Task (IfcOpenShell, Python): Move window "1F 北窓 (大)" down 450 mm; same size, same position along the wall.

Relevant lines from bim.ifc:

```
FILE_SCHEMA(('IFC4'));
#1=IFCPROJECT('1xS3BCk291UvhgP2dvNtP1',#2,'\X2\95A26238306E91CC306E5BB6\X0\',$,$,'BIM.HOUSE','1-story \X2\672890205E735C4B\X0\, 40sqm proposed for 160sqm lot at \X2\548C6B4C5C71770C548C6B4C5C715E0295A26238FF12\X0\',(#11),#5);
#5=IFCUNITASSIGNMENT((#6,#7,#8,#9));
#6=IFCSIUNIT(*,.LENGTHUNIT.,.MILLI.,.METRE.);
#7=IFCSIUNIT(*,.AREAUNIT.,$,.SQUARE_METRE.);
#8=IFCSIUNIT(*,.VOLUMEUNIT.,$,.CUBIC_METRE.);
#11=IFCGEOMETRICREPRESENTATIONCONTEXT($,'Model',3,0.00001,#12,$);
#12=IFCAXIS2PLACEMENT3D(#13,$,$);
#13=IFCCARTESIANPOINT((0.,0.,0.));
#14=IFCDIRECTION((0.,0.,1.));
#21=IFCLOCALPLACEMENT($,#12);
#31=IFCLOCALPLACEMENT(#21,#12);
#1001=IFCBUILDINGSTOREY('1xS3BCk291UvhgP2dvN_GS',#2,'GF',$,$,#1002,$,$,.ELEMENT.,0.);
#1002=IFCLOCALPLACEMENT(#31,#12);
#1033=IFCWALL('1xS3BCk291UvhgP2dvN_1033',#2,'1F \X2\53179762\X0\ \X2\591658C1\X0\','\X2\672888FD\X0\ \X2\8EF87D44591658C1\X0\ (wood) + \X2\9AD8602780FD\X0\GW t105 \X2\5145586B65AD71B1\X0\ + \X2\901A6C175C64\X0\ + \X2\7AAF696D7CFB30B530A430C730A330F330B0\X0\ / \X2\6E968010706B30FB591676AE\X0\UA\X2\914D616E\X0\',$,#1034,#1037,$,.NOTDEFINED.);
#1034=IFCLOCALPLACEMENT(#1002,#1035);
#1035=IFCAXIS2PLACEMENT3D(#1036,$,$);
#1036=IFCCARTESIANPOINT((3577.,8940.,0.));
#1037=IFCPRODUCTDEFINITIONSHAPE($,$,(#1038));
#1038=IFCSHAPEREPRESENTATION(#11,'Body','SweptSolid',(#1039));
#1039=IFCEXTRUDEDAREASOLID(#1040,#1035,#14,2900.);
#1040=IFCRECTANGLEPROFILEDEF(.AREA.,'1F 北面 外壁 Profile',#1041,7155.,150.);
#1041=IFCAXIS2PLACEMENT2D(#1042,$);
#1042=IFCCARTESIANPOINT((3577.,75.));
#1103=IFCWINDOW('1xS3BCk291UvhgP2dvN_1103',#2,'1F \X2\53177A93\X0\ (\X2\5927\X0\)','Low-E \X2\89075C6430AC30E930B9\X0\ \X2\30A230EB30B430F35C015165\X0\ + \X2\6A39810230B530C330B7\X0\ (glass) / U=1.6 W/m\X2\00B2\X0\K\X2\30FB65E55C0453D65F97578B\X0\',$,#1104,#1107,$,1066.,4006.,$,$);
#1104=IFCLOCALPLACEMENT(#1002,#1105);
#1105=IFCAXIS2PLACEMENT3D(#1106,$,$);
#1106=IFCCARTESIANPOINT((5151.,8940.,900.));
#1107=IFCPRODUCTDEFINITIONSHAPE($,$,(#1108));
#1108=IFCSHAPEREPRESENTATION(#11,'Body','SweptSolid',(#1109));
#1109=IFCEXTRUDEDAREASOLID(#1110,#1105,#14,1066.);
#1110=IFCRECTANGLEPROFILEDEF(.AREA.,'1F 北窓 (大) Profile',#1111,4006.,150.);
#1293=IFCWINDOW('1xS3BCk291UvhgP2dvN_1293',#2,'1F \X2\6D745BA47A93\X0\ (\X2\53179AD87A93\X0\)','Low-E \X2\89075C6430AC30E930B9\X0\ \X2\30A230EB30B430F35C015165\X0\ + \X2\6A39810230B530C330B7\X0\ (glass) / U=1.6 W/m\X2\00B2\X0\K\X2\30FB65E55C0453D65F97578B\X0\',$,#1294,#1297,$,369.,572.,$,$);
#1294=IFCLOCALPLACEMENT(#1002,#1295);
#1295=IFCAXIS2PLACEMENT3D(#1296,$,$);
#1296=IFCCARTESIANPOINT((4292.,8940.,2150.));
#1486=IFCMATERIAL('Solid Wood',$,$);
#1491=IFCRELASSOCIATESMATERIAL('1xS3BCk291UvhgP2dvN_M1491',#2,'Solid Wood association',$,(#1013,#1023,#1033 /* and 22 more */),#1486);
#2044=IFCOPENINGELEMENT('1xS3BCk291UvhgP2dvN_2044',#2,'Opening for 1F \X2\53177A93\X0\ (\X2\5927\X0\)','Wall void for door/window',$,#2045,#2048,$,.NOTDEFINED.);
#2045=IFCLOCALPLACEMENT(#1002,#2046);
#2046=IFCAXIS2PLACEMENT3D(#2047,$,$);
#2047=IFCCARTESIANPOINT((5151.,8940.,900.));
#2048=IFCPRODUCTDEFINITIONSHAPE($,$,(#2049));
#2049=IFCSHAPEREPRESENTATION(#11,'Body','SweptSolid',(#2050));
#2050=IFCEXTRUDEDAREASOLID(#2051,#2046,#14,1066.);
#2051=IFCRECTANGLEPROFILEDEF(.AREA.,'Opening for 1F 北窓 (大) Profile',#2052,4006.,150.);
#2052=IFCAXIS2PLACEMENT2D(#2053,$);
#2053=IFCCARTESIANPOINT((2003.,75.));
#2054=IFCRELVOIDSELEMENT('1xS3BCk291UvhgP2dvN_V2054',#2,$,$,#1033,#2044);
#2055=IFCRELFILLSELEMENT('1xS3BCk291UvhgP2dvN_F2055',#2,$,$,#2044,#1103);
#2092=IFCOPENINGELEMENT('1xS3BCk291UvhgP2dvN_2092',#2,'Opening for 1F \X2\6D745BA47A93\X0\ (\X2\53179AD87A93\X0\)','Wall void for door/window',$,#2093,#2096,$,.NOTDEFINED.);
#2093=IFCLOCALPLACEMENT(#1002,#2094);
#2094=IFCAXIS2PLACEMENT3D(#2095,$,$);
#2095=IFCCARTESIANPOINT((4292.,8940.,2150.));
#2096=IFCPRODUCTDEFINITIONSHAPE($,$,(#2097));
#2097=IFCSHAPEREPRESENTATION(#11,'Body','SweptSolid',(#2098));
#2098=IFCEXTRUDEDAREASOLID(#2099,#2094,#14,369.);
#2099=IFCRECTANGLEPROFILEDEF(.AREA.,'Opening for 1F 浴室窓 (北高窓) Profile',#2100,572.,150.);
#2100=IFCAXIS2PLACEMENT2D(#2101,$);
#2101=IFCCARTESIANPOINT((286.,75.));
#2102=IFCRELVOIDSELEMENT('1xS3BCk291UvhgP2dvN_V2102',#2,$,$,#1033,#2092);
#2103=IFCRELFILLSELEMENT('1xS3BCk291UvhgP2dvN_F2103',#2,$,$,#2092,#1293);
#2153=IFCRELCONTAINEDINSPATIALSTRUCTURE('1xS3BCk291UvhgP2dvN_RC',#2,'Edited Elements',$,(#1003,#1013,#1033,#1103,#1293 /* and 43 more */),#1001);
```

```python
import numpy as np
import ifcopenshell
import ifcopenshell.api.geometry
import ifcopenshell.util.placement
import ifcopenshell.util.unit

model = ifcopenshell.open("bim.ifc")
unit_scale = ifcopenshell.util.unit.calculate_unit_scale(model)

window = model.by_id(1103)
opening = window.FillsVoids[0].RelatingOpeningElement
dz = -0.45 / unit_scale

shift = np.array([0.0, 0.0, dz])
# The window is not placed relative to its opening, so move both.
for product in (opening, window):
    matrix = ifcopenshell.util.placement.get_local_placement(product.ObjectPlacement)
    matrix[:3, 3] += shift
    ifcopenshell.api.geometry.edit_object_placement(model, product=product, matrix=matrix, is_si=False)

print(f"moved by {dz * unit_scale:+.3f} m")

model.write("bim-out.ifc")
```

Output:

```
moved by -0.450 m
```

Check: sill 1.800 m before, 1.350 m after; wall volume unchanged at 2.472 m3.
